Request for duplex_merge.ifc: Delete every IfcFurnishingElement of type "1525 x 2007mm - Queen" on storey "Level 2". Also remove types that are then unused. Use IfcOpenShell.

First a look at what the model holds.

```python
import ifcopenshell
import ifcopenshell.util.element

model = ifcopenshell.open("duplex_merge.ifc")
print(model.schema)
storey = next(s for s in model.by_type("IfcBuildingStorey") if s.Name == "Level 2")
furniture = [e for e in ifcopenshell.util.element.get_decomposition(storey) if e.is_a("IfcFurnishingElement")]
seen = {}
for e in furniture:
    element_type = ifcopenshell.util.element.get_type(e)
    name = element_type.Name if element_type not in (None, e) else None
    seen[name] = seen.get(name, 0) + 1
for name, count in sorted(seen.items(), key=str):
    print(count, "x", name)
```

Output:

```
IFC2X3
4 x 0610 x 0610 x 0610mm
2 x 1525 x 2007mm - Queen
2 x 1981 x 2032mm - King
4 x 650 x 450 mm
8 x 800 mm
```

```python
import ifcopenshell
import ifcopenshell.api.root
import ifcopenshell.util.element

model = ifcopenshell.open("duplex_merge.ifc")

storey = next(s for s in model.by_type("IfcBuildingStorey") if s.Name == "Level 2")
furniture = [e for e in ifcopenshell.util.element.get_decomposition(storey) if e.is_a("IfcFurnishingElement")]
targets = [e for e in furniture if (t := ifcopenshell.util.element.get_type(e)) not in (None, e) and t.Name == "1525 x 2007mm - Queen"]
types = {ifcopenshell.util.element.get_type(e) for e in targets} - {None, *targets}

for e in targets:
    ifcopenshell.api.root.remove_product(model, product=e)
print(len(targets), "removed")

unused = [t for t in types if not ifcopenshell.util.element.get_types(t)]
for t in unused:
    ifcopenshell.api.root.remove_product(model, product=t)
print(len(unused), "unused types removed")

model.write("duplex_merge_rev.ifc")
```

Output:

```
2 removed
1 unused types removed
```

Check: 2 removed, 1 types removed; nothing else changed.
